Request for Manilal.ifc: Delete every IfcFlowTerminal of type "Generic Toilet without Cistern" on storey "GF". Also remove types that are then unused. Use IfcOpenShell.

First a look at what the model holds.

```python
import ifcopenshell
import ifcopenshell.util.element

model = ifcopenshell.open("Manilal.ifc")
print(model.schema)
storey = next(s for s in model.by_type("IfcBuildingStorey") if s.Name == "GF")
terminals = [e for e in ifcopenshell.util.element.get_decomposition(storey) if e.is_a("IfcFlowTerminal")]
seen = {}
for e in terminals:
    element_type = ifcopenshell.util.element.get_type(e)
    name = element_type.Name if element_type not in (None, e) else None
    seen[name] = seen.get(name, 0) + 1
for name, count in sorted(seen.items(), key=str):
    print(count, "x", name)
```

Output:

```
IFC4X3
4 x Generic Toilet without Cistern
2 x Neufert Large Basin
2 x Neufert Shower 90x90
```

```python
import ifcopenshell
import ifcopenshell.api.root
import ifcopenshell.util.element

model = ifcopenshell.open("Manilal.ifc")

storey = next(s for s in model.by_type("IfcBuildingStorey") if s.Name == "GF")
terminals = [e for e in ifcopenshell.util.element.get_decomposition(storey) if e.is_a("IfcFlowTerminal")]
targets = [e for e in terminals if (t := ifcopenshell.util.element.get_type(e)) not in (None, e) and t.Name == "Generic Toilet without Cistern"]
types = {ifcopenshell.util.element.get_type(e) for e in targets} - {None, *targets}

for e in targets:
    ifcopenshell.api.root.remove_product(model, product=e)
print(len(targets), "removed")

unused = [t for t in types if not ifcopenshell.util.element.get_types(t)]
for t in unused:
    ifcopenshell.api.root.remove_product(model, product=t)
print(len(unused), "unused types removed")

model.write("Manilal_edited.ifc")
```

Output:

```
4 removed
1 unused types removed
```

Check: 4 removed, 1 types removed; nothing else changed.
